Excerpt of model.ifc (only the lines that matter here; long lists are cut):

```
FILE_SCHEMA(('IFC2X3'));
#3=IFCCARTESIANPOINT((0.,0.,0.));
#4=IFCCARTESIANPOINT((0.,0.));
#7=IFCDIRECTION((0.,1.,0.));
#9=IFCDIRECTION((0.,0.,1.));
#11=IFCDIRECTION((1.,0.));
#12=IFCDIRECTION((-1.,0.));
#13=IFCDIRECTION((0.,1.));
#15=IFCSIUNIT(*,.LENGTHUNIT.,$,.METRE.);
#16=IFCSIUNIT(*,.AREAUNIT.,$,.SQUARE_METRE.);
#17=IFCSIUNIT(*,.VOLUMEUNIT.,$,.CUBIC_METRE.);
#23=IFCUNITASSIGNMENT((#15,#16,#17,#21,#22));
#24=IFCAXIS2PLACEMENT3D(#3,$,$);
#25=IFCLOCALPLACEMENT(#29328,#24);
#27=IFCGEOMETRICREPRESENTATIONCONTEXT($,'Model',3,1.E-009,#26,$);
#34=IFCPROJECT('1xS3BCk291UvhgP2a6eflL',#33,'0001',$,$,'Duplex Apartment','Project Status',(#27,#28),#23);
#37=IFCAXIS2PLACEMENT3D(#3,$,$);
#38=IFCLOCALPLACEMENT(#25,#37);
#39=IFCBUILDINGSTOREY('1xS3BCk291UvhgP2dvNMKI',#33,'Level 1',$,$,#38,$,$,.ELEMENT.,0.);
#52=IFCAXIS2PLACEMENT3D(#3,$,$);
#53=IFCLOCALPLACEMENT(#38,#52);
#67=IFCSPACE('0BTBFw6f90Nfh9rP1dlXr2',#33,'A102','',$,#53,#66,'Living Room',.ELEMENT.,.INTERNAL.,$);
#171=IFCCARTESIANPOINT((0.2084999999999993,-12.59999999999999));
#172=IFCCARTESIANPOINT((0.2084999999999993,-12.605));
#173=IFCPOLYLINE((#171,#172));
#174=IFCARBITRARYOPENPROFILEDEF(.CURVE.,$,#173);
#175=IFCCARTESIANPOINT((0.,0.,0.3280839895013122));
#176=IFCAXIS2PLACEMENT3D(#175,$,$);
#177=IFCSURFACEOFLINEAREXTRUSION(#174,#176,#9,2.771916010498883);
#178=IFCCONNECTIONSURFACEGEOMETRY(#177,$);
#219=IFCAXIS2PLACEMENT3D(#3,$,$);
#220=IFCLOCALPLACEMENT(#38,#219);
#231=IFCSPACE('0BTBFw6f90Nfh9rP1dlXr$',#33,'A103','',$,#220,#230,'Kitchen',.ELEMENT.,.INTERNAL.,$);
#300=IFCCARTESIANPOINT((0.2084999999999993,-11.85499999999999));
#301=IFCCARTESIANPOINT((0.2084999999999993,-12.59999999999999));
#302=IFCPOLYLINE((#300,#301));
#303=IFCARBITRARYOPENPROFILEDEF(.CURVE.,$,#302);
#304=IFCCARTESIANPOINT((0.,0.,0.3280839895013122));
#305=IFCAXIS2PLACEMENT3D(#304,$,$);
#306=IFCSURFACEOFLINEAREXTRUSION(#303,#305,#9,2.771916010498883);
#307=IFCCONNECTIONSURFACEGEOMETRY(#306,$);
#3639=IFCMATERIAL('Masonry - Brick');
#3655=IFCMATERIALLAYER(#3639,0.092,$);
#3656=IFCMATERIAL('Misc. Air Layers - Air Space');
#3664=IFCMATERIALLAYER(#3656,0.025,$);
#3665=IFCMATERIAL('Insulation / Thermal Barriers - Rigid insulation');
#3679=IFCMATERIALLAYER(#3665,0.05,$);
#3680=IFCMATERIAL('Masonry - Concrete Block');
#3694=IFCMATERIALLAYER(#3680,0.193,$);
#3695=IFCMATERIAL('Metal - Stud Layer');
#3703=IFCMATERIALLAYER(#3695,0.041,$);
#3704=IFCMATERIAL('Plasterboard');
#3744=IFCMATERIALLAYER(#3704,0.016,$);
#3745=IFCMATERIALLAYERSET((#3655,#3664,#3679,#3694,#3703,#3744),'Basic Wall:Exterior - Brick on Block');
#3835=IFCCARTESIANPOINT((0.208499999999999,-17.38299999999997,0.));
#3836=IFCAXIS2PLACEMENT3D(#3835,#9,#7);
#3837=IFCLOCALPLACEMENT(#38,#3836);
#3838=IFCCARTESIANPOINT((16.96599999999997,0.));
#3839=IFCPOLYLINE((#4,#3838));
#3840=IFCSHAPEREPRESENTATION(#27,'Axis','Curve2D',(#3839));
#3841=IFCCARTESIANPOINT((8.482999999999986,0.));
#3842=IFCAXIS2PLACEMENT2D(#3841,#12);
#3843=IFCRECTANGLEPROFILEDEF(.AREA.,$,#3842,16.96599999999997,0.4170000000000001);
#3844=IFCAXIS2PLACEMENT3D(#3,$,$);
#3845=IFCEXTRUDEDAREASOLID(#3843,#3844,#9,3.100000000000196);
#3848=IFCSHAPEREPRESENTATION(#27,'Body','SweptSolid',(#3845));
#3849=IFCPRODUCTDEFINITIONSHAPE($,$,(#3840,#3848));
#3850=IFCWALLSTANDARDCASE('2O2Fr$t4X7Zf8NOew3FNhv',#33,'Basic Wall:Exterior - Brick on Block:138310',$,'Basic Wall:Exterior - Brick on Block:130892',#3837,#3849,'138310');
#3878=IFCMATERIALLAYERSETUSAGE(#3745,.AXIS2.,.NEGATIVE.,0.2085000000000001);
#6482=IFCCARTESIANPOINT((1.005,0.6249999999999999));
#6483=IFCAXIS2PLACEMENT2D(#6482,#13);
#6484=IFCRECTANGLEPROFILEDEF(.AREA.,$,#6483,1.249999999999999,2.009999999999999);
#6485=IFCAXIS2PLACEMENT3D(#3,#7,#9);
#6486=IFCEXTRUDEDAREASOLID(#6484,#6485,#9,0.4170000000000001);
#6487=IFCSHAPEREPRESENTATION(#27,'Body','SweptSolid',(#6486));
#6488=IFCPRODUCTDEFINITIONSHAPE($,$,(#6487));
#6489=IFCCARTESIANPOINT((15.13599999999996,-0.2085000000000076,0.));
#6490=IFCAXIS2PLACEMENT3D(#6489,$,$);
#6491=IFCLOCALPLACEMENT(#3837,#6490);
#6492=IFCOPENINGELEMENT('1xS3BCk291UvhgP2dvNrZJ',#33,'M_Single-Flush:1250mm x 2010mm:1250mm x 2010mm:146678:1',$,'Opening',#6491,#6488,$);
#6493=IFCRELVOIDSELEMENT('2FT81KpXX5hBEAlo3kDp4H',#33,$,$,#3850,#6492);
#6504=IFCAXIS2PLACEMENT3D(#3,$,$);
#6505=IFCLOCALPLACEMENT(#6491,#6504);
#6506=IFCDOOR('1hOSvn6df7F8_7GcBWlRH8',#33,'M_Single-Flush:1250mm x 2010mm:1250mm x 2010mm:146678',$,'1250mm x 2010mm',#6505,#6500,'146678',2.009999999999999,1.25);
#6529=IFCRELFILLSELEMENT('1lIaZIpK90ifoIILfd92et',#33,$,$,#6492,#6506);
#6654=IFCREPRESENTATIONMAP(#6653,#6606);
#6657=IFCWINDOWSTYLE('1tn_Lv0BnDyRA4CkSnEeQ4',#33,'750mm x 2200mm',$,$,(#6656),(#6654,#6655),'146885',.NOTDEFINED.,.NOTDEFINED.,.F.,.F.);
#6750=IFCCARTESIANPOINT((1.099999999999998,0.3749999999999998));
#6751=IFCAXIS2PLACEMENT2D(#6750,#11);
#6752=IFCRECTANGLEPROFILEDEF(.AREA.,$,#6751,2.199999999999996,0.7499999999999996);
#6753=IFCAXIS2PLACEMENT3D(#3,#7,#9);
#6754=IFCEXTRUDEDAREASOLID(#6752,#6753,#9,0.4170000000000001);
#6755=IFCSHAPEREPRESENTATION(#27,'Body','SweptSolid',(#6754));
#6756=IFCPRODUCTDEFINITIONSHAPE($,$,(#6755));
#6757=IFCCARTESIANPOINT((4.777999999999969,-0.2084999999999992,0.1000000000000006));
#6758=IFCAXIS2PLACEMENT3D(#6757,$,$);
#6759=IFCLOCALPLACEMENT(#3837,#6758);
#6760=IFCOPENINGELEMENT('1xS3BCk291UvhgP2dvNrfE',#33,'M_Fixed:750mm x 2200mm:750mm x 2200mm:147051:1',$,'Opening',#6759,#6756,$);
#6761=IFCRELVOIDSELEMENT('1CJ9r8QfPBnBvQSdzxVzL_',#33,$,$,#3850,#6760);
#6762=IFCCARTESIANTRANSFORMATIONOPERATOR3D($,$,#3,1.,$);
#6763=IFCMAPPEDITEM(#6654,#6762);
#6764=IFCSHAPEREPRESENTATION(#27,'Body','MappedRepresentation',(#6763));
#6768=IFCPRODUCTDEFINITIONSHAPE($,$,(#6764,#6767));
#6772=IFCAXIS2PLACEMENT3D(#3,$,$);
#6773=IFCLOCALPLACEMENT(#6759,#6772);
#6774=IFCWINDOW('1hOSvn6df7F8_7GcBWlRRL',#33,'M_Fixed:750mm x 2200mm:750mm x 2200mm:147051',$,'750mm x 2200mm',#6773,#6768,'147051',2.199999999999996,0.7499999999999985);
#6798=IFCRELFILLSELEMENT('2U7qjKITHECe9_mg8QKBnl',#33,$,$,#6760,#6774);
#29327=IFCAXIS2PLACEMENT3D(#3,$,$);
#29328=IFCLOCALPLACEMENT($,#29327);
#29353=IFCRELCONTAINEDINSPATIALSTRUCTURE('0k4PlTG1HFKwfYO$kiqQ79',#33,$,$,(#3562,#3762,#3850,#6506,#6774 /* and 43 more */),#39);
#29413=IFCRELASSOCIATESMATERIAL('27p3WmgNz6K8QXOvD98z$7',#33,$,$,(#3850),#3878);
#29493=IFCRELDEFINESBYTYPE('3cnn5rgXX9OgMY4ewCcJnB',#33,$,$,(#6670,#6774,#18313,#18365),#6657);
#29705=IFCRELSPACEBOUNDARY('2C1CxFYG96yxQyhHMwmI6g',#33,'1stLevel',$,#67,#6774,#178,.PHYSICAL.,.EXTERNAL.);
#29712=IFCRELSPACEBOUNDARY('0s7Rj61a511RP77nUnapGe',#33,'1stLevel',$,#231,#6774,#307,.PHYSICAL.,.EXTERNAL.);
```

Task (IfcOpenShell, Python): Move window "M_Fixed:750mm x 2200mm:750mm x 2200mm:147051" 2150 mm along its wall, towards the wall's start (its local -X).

```python
import numpy as np
import ifcopenshell
import ifcopenshell.api.geometry
import ifcopenshell.util.placement
import ifcopenshell.util.unit

model = ifcopenshell.open("model.ifc")
unit_scale = ifcopenshell.util.unit.calculate_unit_scale(model)

window = model.by_guid("1hOSvn6df7F8_7GcBWlRRL")
opening = window.FillsVoids[0].RelatingOpeningElement
wall = opening.VoidsElements[0].RelatingBuildingElement

wall_matrix = ifcopenshell.util.placement.get_local_placement(wall.ObjectPlacement)
shift = wall_matrix[:3, 0] * -2.15 / unit_scale
before = ifcopenshell.util.placement.get_local_placement(window.ObjectPlacement)[:3, 3].copy()

# The window is placed relative to its opening, so it follows when the opening moves.
matrix = ifcopenshell.util.placement.get_local_placement(opening.ObjectPlacement)
matrix[:3, 3] += shift
ifcopenshell.api.geometry.edit_object_placement(
    model, product=opening, matrix=matrix, is_si=False, should_transform_children=True
)

# Space boundary surfaces are stored in each space's coordinates; move them too.
for rel in window.ProvidesBoundaries:
    if not rel.ConnectionGeometry:
        continue
    surface = rel.ConnectionGeometry.SurfaceOnRelatingElement
    space_matrix = ifcopenshell.util.placement.get_local_placement(rel.RelatingSpace.ObjectPlacement)
    point = np.array(surface.Position.Location.Coordinates) + space_matrix[:3, :3].T @ shift
    surface.Position = model.createIfcAxis2Placement3D(
        model.createIfcCartesianPoint(point.tolist()), surface.Position.Axis, surface.Position.RefDirection
    )

after = ifcopenshell.util.placement.get_local_placement(window.ObjectPlacement)[:3, 3]
print("window moved by", (after - before).round(3) + 0.0)

model.write("model_v2.ifc")
```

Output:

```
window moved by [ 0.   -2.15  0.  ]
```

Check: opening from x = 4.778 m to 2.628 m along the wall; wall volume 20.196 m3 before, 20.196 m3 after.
